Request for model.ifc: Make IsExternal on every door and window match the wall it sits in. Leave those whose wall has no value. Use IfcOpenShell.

First a look at what the model holds.

```python
import ifcopenshell
import ifcopenshell.util.element

model = ifcopenshell.open("model.ifc")
print(model.schema)
seen = {}
for e in model.by_type("IfcDoor") + model.by_type("IfcWindow"):
    if not e.FillsVoids:
        continue
    host = e.FillsVoids[0].RelatingOpeningElement.VoidsElements[0].RelatingBuildingElement
    own = ifcopenshell.util.element.get_pset(e, f"Pset_{e.is_a()[3:].removesuffix('StandardCase')}Common", "IsExternal")
    wall = ifcopenshell.util.element.get_pset(host, "Pset_WallCommon", "IsExternal")
    seen[e.is_a(), own, wall] = seen.get((e.is_a(), own, wall), 0) + 1
for (cls, own, wall), count in sorted(seen.items(), key=str):
    print(count, cls, "IsExternal:", own, "| host wall:", wall)
```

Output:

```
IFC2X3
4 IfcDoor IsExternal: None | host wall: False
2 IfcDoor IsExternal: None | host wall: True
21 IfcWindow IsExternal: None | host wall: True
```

```python
import ifcopenshell
import ifcopenshell.api.pset
import ifcopenshell.util.element

model = ifcopenshell.open("model.ifc")

count = 0
for ifc_class, pset_name in (("IfcDoor", "Pset_DoorCommon"), ("IfcWindow", "Pset_WindowCommon")):
    for e in model.by_type(ifc_class):
        if not e.FillsVoids:
            continue
        host = e.FillsVoids[0].RelatingOpeningElement.VoidsElements[0].RelatingBuildingElement
        external = ifcopenshell.util.element.get_pset(host, "Pset_WallCommon", "IsExternal")
        if external is None or ifcopenshell.util.element.get_pset(e, pset_name, "IsExternal") == external:
            continue
        pset = ifcopenshell.api.pset.add_pset(model, product=e, name=pset_name)
        ifcopenshell.api.pset.edit_pset(model, pset=pset, properties={"IsExternal": external})
        count += 1

print(count, "updated")

model.write("model-out.ifc")
```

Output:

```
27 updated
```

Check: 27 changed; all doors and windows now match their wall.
